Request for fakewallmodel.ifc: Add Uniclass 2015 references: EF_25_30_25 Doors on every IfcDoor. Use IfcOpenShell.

First a look at what the model holds.

```python
import ifcopenshell

model = ifcopenshell.open("fakewallmodel.ifc")
print(model.schema)
print("classifications:", [c.Name for c in model.by_type("IfcClassification")])
for ifc_class in ("IfcDoor", "IfcRoof", "IfcStair", "IfcWall", "IfcWindow"):
    print(ifc_class, len(model.by_type(ifc_class)))
```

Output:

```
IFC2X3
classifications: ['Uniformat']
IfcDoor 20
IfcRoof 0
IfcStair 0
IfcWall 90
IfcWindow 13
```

```python
import ifcopenshell
import ifcopenshell.api.classification

model = ifcopenshell.open("fakewallmodel.ifc")

# IFC2X3 requires Source and Edition and has no link from the project to the system.
system = model.create_entity("IfcClassification", Source="NBS", Edition="2015", Name="Uniclass 2015")

codes = {
    "IfcDoor": ("EF_25_30_25", "Doors"),
}
for ifc_class, (code, name) in codes.items():
    products = model.by_type(ifc_class)
    ifcopenshell.api.classification.add_reference(
        model, products=products, classification=system, identification=code, name=name
    )
    print(code, len(products))

model.write("fakewallmodel_updated.ifc")
```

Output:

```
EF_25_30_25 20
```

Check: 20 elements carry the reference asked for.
